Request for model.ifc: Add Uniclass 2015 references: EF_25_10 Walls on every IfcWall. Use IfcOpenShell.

First a look at what the model holds.

```python
import ifcopenshell

model = ifcopenshell.open("model.ifc")
print(model.schema)
print("classifications:", [c.Name for c in model.by_type("IfcClassification")])
for ifc_class in ("IfcDoor", "IfcRoof", "IfcStair", "IfcWall", "IfcWindow"):
    print(ifc_class, len(model.by_type(ifc_class)))
```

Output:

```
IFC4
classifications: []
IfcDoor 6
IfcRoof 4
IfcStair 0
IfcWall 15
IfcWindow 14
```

```python
import ifcopenshell
import ifcopenshell.api.classification

model = ifcopenshell.open("model.ifc")

system = ifcopenshell.api.classification.add_classification(model, classification="Uniclass 2015")

codes = {
    "IfcWall": ("EF_25_10", "Walls"),
}
for ifc_class, (code, name) in codes.items():
    products = model.by_type(ifc_class)
    ifcopenshell.api.classification.add_reference(
        model, products=products, classification=system, identification=code, name=name
    )
    print(code, len(products))

model.write("model_edited.ifc")
```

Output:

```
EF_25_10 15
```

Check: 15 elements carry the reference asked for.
